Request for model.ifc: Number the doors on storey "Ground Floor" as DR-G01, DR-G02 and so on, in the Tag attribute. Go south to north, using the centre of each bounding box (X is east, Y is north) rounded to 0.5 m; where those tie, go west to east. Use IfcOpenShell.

First a look at what the model holds.

```python
import ifcopenshell
import ifcopenshell.util.element
import ifcopenshell.util.placement

model = ifcopenshell.open("model.ifc")
print(model.schema)
storey = next(s for s in model.by_type("IfcBuildingStorey") if s.Name == "Ground Floor")
doors = [e for e in ifcopenshell.util.element.get_decomposition(storey) if e.is_a("IfcDoor")]
for e in sorted(doors, key=lambda e: e.id()):
    origin = ifcopenshell.util.placement.get_local_placement(e.ObjectPlacement)[:3, 3]
    print(e.id(), e.Tag, e.Name, origin.round(2) + 0.0, sep=" | ")
```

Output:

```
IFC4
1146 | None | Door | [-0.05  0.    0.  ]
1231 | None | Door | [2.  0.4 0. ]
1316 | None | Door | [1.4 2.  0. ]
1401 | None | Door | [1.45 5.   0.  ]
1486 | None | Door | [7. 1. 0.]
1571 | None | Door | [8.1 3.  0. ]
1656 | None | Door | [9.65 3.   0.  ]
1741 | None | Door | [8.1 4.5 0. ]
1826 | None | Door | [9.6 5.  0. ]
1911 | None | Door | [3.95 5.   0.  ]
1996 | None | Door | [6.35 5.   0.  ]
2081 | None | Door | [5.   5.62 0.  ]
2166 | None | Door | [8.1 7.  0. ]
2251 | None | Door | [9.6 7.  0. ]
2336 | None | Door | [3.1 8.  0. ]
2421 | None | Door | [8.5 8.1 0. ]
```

```python
import ifcopenshell
import ifcopenshell.geom
import ifcopenshell.util.element
import ifcopenshell.util.shape

model = ifcopenshell.open("model.ifc")
settings = ifcopenshell.geom.settings()
settings.set("use-world-coords", True)


def centre(element):
    shape = ifcopenshell.geom.create_shape(settings, element)
    return ifcopenshell.util.shape.get_bbox_centroid(shape.geometry)


storey = next(s for s in model.by_type("IfcBuildingStorey") if s.Name == "Ground Floor")
doors = [e for e in ifcopenshell.util.element.get_decomposition(storey) if e.is_a("IfcDoor")]

# Insertion points can sit at a corner or the storey origin, so sort by the geometry (in metres).
centres = {e: centre(e) for e in doors}
doors.sort(key=lambda e: (round(centres[e][1] / 0.5), centres[e][0]))

for i, e in enumerate(doors, start=1):
    number = f"DR-G{i:02d}"
    e.Tag = number
    print(e.id(), number)

model.write("model_rev.ifc")
```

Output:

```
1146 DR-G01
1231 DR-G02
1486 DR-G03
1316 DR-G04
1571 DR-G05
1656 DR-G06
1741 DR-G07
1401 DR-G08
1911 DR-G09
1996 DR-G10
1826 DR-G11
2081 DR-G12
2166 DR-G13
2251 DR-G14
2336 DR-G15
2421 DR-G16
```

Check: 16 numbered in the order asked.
